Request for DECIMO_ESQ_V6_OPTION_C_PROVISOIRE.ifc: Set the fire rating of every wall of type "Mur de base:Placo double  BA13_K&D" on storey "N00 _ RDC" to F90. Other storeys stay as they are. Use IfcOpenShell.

First a look at what the model holds.

```python
import ifcopenshell
import ifcopenshell.util.element

model = ifcopenshell.open("DECIMO_ESQ_V6_OPTION_C_PROVISOIRE.ifc")
print(model.schema)
storey = next(s for s in model.by_type("IfcBuildingStorey") if s.Name == "N00 _ RDC")
walls = [e for e in ifcopenshell.util.element.get_decomposition(storey) if e.is_a("IfcWall")]
seen = {}
for e in walls:
    element_type = ifcopenshell.util.element.get_type(e)
    key = (element_type.Name if element_type != e and element_type else None, ifcopenshell.util.element.get_pset(e, "Pset_WallCommon", "FireRating"))
    seen[key] = seen.get(key, 0) + 1
for (name, value), count in sorted(seen.items(), key=str):
    print(count, "x", name, "|", value)
```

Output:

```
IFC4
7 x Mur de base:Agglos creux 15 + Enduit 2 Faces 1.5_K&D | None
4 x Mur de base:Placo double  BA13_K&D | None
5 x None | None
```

```python
import ifcopenshell
import ifcopenshell.api.pset
import ifcopenshell.util.element

model = ifcopenshell.open("DECIMO_ESQ_V6_OPTION_C_PROVISOIRE.ifc")

storey = next(s for s in model.by_type("IfcBuildingStorey") if s.Name == "N00 _ RDC")
walls = [e for e in ifcopenshell.util.element.get_decomposition(storey) if e.is_a("IfcWall")]

count = 0
for e in walls:
    element_type = ifcopenshell.util.element.get_type(e)
    if element_type in (None, e) or element_type.Name != "Mur de base:Placo double  BA13_K&D":
        continue
    # add_pset returns the element's existing set when there is one.
    pset = ifcopenshell.api.pset.add_pset(model, product=e, name="Pset_WallCommon")
    ifcopenshell.api.pset.edit_pset(model, pset=pset, properties={"FireRating": "F90"})
    count += 1

print(count, "walls updated")

model.write("DECIMO_ESQ_V6_OPTION_C_PROVISOIRE-out.ifc")
```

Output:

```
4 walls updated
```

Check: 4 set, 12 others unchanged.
